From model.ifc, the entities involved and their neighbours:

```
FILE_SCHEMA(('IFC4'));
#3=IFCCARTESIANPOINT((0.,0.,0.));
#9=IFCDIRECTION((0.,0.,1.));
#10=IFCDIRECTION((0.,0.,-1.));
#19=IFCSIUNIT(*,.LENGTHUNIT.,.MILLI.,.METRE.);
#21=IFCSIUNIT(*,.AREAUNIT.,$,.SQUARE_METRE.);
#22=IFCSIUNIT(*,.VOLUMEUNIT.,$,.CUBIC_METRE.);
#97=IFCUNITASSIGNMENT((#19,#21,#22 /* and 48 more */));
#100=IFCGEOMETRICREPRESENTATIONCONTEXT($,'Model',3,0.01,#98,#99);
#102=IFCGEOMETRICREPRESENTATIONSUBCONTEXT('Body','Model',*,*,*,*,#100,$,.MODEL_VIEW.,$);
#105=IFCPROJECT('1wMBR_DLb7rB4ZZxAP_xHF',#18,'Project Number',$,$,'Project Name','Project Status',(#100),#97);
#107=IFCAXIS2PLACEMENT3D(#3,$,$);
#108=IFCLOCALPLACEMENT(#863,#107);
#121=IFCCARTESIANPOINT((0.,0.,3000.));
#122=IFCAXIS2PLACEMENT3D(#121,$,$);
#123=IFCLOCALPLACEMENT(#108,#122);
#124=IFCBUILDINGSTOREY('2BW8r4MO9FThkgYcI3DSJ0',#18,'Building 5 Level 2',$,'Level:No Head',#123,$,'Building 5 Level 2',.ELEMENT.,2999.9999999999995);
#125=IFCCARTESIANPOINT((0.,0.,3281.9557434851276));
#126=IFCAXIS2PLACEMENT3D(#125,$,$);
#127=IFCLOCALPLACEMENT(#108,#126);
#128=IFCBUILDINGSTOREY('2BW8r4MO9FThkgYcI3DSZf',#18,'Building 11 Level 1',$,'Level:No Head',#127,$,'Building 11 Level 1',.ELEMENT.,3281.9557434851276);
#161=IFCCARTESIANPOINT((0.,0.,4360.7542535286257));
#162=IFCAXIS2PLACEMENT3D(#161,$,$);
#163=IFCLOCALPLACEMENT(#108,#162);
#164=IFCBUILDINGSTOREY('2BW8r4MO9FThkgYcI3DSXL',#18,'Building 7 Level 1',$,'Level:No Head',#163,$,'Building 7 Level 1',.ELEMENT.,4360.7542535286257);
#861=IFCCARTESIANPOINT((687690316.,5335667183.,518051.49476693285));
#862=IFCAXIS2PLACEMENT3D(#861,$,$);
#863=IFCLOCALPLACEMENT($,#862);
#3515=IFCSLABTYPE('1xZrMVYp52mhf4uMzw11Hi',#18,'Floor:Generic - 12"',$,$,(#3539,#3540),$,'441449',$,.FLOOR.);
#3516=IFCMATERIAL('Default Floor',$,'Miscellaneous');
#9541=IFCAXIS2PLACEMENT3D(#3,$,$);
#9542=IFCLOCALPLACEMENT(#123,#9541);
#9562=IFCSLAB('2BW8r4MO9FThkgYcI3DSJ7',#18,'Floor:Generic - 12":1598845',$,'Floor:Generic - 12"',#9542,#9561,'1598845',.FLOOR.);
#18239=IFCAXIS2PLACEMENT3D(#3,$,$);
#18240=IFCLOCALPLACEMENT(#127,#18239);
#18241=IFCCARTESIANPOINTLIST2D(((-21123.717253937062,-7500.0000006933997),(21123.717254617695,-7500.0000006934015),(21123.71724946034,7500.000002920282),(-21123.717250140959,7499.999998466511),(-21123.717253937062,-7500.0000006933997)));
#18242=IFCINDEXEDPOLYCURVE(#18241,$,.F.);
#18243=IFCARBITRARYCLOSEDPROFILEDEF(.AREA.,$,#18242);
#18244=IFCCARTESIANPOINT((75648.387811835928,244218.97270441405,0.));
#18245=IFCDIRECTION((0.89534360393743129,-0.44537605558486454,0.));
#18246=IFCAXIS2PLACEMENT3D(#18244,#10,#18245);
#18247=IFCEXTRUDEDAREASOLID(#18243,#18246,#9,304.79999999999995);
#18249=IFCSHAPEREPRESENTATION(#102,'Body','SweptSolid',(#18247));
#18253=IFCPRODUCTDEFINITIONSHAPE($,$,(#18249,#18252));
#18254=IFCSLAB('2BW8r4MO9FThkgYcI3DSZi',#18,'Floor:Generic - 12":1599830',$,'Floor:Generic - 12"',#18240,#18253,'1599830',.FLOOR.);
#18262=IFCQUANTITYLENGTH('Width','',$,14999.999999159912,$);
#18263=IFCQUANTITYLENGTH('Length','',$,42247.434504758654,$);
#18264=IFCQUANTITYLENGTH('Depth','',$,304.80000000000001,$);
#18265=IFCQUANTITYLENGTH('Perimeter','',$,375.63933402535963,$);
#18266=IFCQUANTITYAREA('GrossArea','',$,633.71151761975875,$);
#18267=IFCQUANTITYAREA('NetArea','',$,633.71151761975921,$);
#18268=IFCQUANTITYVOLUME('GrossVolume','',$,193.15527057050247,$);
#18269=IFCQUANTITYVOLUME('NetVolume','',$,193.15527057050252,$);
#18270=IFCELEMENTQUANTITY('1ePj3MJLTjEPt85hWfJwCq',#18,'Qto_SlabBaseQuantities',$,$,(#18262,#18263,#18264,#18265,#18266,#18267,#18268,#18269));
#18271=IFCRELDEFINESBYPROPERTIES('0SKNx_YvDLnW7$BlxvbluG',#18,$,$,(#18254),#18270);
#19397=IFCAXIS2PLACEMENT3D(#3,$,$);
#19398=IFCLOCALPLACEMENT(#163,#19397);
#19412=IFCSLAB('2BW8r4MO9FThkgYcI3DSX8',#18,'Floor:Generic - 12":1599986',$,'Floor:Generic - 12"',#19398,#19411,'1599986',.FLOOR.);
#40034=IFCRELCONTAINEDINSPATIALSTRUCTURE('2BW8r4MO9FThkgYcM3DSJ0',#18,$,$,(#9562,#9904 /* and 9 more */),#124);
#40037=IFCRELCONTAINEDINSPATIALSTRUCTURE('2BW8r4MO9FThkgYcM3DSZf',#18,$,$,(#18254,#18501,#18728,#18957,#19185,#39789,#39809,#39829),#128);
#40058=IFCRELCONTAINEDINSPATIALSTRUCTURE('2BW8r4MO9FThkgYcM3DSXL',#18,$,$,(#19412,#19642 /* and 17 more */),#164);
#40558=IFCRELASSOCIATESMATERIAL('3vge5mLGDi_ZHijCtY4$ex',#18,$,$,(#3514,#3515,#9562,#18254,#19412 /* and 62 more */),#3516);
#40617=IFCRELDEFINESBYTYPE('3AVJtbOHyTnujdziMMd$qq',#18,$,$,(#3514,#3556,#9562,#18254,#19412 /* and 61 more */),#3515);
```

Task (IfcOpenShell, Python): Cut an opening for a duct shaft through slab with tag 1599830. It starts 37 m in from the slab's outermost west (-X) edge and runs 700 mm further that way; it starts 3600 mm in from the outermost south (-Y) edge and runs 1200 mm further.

```python
import numpy as np
import ifcopenshell
import ifcopenshell.api.feature
import ifcopenshell.api.geometry
import ifcopenshell.api.pset
import ifcopenshell.api.root
import ifcopenshell.geom
import ifcopenshell.util.element
import ifcopenshell.util.placement
import ifcopenshell.util.representation
import ifcopenshell.util.shape
import ifcopenshell.util.unit

model = ifcopenshell.open("model.ifc")
unit_scale = ifcopenshell.util.unit.calculate_unit_scale(model)
area_scale = ifcopenshell.util.unit.calculate_unit_scale(model, "AREAUNIT")
volume_scale = ifcopenshell.util.unit.calculate_unit_scale(model, "VOLUMEUNIT")
settings = ifcopenshell.geom.settings()


def volume(element):
    """Net volume in cubic metres, openings subtracted."""
    shape = ifcopenshell.geom.create_shape(settings, element)
    return ifcopenshell.util.shape.get_volume(shape.geometry)


slab = model.by_guid("2BW8r4MO9FThkgYcI3DSZi")
before = volume(slab)

# Extent in the slab's own axes, in metres. The edges named are its -X and -Y sides.
slab_shape = ifcopenshell.geom.create_shape(settings, slab)
vertices = ifcopenshell.util.shape.get_vertices(slab_shape.geometry)
x_min, y_min, bottom = vertices.min(axis=0)
top = vertices[:, 2].max()

opening = ifcopenshell.api.root.create_entity(model, ifc_class="IfcOpeningElement", name="Duct shaft opening", predefined_type="OPENING")
context = ifcopenshell.util.representation.get_context(model, "Model", "Body", "MODEL_VIEW")
width, depth = 0.7, 1.2
outline = [(0.0, 0.0), (width, 0.0), (width, depth), (0.0, depth), (0.0, 0.0)]
# Overshoot both faces by 50 mm so the cut is clean.
shape = ifcopenshell.api.geometry.add_slab_representation(
    model, context=context, depth=top - bottom + 0.1, polyline=outline
)
ifcopenshell.api.geometry.assign_representation(model, product=opening, representation=shape)

matrix = ifcopenshell.util.placement.get_local_placement(slab.ObjectPlacement)
matrix[:, 3] = matrix @ np.append(np.array([x_min + 37, y_min + 3.6, bottom - 0.05]) / unit_scale, 1.0)
ifcopenshell.api.geometry.edit_object_placement(model, product=opening, matrix=matrix, is_si=False)
ifcopenshell.api.feature.add_feature(model, feature=opening, element=slab)

after = volume(slab)

# Update the slab's stored quantities.
qto = model.by_id(ifcopenshell.util.element.get_pset(slab, "Qto_SlabBaseQuantities", should_inherit=False)["id"])
ifcopenshell.api.pset.edit_qto(model, qto=qto, properties={
    "NetArea": after / (top - bottom) / area_scale,
    "NetVolume": after / volume_scale,
})

print(f"slab volume {before:.3f} -> {after:.3f} m3")

model.write("model_updated.ifc")
```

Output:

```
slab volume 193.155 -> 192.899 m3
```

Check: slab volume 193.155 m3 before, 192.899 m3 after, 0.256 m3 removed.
